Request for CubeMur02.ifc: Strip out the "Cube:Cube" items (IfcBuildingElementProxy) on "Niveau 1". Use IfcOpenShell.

First a look at what the model holds.

```python
import ifcopenshell
import ifcopenshell.util.element

model = ifcopenshell.open("CubeMur02.ifc")
print(model.schema)
storey = next(s for s in model.by_type("IfcBuildingStorey") if s.Name == "Niveau 1")
proxies = [e for e in ifcopenshell.util.element.get_decomposition(storey) if e.is_a("IfcBuildingElementProxy")]
seen = {}
for e in proxies:
    element_type = ifcopenshell.util.element.get_type(e)
    name = element_type.Name if element_type not in (None, e) else None
    seen[name] = seen.get(name, 0) + 1
for name, count in sorted(seen.items(), key=str):
    print(count, "x", name)
```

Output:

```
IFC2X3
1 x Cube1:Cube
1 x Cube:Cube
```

```python
import ifcopenshell
import ifcopenshell.api.root
import ifcopenshell.util.element

model = ifcopenshell.open("CubeMur02.ifc")

storey = next(s for s in model.by_type("IfcBuildingStorey") if s.Name == "Niveau 1")
proxies = [e for e in ifcopenshell.util.element.get_decomposition(storey) if e.is_a("IfcBuildingElementProxy")]
targets = [e for e in proxies if (t := ifcopenshell.util.element.get_type(e)) not in (None, e) and t.Name == "Cube:Cube"]

for e in targets:
    ifcopenshell.api.root.remove_product(model, product=e)
print(len(targets), "removed")

model.write("CubeMur02-out.ifc")
```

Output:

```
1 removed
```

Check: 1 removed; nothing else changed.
